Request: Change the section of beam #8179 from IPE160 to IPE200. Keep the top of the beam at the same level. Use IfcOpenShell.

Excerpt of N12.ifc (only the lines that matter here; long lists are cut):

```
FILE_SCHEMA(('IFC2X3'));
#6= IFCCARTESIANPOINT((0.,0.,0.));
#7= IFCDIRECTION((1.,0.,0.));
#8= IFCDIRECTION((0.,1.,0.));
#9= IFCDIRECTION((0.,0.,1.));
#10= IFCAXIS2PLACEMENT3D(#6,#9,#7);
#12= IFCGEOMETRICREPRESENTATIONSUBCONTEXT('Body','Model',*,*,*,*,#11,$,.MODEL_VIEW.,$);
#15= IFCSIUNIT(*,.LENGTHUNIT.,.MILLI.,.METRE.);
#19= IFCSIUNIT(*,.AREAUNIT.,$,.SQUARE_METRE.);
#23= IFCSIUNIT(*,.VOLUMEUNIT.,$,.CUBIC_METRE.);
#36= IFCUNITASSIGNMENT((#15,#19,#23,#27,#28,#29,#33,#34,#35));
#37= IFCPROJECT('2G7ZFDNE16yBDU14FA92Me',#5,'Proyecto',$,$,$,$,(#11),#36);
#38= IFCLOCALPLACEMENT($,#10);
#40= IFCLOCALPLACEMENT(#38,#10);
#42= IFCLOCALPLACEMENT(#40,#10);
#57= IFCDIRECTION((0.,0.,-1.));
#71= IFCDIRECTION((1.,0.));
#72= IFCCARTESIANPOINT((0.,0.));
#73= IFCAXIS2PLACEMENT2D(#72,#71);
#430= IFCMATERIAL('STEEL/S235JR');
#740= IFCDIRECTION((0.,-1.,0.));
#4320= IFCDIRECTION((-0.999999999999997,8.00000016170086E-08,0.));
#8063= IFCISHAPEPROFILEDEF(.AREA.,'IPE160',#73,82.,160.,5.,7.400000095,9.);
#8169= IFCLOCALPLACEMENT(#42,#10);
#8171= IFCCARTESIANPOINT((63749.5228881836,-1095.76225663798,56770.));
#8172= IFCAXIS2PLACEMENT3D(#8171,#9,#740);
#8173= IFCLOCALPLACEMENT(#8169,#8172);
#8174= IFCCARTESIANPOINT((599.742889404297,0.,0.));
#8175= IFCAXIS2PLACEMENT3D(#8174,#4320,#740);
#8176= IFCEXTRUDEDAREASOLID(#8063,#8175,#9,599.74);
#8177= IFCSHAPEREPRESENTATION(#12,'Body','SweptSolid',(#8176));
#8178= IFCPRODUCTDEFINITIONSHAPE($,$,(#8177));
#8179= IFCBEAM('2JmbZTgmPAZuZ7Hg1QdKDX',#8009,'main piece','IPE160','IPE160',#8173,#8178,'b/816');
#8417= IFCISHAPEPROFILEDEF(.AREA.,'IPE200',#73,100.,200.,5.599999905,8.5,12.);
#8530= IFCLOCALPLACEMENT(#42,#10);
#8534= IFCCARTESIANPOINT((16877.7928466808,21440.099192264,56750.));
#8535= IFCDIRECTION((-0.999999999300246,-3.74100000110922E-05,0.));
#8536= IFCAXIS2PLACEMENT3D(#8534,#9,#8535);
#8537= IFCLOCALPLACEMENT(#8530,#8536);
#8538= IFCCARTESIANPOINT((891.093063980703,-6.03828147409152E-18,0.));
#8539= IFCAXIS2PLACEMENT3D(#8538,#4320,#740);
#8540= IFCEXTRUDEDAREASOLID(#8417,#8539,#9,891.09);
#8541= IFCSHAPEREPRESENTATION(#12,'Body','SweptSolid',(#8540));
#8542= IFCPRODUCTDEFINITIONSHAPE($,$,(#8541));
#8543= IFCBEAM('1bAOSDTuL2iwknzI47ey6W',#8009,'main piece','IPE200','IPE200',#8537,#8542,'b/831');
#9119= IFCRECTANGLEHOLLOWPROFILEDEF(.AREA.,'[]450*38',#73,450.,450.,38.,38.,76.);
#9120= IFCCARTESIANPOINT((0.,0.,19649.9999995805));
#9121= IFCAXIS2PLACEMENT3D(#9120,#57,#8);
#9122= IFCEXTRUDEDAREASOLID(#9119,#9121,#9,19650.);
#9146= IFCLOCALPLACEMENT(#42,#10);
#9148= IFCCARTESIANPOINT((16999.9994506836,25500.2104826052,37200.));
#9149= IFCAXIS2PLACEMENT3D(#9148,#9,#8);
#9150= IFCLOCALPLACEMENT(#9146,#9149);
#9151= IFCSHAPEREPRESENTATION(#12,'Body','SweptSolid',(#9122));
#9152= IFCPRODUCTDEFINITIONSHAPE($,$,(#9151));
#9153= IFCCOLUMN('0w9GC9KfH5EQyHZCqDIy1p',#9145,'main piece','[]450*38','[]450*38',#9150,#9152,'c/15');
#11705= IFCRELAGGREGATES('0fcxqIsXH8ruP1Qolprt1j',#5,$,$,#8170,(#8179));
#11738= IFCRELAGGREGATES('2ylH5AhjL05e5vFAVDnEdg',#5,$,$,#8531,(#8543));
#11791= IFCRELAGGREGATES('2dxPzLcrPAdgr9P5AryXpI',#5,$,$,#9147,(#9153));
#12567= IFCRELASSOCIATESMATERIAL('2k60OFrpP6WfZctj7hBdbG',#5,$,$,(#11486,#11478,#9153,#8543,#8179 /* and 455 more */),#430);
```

```python
import ifcopenshell
import ifcopenshell.util.element
import ifcopenshell.util.representation

model = ifcopenshell.open("N12.ifc")

member = model.by_id(8179)
source = next(p for p in model.by_type("IfcIShapeProfileDef") if p.ProfileName == "IPE200")

body = ifcopenshell.util.representation.get_representation(member, "Model", "Body")
solid = body.Items[0]
old_profile = solid.SweptArea

# Copy the section's sizes but keep this member's own profile position.
profile = ifcopenshell.util.element.copy(model, source)
# Profiles are centred, so shift by half the change in depth to hold the top.
shift = (old_profile.OverallDepth - profile.OverallDepth) / 2
x, y = old_profile.Position.Location.Coordinates
up = (0.0, 1.0)  # upwards, in the solid's own plane
location = model.createIfcCartesianPoint((x + up[0] * shift, y + up[1] * shift))
profile.Position = model.createIfcAxis2Placement2D(location, old_profile.Position.RefDirection)
solid.SweptArea = profile
if not model.get_total_inverses(old_profile):
    ifcopenshell.util.element.remove_deep2(model, old_profile)
member.Description = member.Description.replace("IPE160", "IPE200")
member.ObjectType = member.ObjectType.replace("IPE160", "IPE200")

print(solid.SweptArea)

model.write("N12_rev.ifc")
```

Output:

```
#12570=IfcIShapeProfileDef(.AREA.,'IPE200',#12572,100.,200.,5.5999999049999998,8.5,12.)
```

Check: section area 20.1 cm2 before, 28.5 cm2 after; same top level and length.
